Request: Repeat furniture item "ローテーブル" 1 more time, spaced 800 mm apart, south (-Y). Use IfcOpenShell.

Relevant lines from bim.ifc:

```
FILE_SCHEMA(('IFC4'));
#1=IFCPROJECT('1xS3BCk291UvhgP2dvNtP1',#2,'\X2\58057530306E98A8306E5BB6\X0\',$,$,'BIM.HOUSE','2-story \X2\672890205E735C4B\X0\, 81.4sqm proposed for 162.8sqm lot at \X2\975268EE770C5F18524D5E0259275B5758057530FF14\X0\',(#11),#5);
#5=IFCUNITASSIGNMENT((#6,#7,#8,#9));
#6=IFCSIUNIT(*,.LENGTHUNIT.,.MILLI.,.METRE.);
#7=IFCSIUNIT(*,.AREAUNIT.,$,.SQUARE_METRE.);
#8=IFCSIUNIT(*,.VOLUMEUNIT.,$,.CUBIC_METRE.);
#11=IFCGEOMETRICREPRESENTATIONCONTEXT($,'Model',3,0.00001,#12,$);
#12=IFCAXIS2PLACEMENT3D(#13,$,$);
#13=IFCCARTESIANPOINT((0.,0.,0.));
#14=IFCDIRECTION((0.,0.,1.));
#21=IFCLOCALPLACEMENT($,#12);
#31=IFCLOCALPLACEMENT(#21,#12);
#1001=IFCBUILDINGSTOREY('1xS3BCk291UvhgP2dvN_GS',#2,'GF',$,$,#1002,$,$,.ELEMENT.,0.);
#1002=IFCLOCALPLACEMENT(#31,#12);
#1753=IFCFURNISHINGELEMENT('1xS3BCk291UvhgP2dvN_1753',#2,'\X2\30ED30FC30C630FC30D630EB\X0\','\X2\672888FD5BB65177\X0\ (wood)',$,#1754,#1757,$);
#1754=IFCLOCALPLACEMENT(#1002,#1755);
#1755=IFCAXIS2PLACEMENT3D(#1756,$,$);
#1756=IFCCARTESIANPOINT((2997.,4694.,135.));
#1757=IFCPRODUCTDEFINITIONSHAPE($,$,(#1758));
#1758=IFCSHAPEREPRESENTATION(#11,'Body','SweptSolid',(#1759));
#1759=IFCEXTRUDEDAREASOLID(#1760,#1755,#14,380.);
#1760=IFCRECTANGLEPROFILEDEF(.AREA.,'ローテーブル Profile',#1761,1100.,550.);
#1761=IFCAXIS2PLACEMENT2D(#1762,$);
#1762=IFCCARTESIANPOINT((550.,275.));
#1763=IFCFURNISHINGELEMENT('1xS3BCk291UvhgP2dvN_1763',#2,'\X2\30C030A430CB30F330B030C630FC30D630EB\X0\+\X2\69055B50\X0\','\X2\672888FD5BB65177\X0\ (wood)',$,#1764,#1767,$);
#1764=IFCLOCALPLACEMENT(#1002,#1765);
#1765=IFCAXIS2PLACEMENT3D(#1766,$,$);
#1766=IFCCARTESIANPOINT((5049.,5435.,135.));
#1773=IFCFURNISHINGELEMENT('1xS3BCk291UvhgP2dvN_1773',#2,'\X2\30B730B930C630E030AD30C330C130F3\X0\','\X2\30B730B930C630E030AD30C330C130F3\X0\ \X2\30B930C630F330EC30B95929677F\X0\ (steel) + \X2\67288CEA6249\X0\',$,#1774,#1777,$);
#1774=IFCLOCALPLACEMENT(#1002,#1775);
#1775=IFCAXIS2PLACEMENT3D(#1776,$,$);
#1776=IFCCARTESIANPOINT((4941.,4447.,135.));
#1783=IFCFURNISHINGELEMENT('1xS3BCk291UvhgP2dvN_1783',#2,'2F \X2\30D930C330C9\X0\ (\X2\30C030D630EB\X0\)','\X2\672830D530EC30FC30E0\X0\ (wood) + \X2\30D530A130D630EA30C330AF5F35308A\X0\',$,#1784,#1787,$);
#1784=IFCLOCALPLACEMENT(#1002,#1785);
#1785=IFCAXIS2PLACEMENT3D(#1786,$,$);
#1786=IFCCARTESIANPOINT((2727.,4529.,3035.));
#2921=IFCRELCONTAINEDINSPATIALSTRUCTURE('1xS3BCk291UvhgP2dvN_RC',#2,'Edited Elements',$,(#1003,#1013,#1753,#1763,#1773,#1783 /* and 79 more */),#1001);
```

```python
import numpy as np
import ifcopenshell
import ifcopenshell.api.geometry
import ifcopenshell.api.root
import ifcopenshell.util.element
import ifcopenshell.util.placement
import ifcopenshell.util.unit

model = ifcopenshell.open("bim.ifc")
unit_scale = ifcopenshell.util.unit.calculate_unit_scale(model)


def reuse_history(source, copy):
    """copy_class also copies each property set's owner history, people and application; keep the originals."""
    for rel in copy.IsDefinedBy:
        if rel.is_a("IfcRelDefinesByProperties") and (history := rel.RelatingPropertyDefinition.OwnerHistory):
            rel.RelatingPropertyDefinition.OwnerHistory = source.OwnerHistory
            ifcopenshell.util.element.remove_deep2(model, history)


source = model.by_guid("1xS3BCk291UvhgP2dvN_1753")
base = ifcopenshell.util.placement.get_local_placement(source.ObjectPlacement)
step = np.array([0.0, -1.0, 0.0]) * 0.8 / unit_scale

for i in range(1, 2):
    copy = ifcopenshell.api.root.copy_class(model, product=source)
    copy.Representation = ifcopenshell.util.element.copy_deep(
        model, source.Representation, exclude=["IfcGeometricRepresentationContext", "IfcRepresentationMap"]
    )
    reuse_history(source, copy)
    matrix = base.copy()
    matrix[:3, 3] += i * step
    print("added at", matrix[:3, 3].round(3) + 0.0)
    ifcopenshell.api.geometry.edit_object_placement(model, product=copy, matrix=matrix, is_si=False)

model.write("bim_updated.ifc")
```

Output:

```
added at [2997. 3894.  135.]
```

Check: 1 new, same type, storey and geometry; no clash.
